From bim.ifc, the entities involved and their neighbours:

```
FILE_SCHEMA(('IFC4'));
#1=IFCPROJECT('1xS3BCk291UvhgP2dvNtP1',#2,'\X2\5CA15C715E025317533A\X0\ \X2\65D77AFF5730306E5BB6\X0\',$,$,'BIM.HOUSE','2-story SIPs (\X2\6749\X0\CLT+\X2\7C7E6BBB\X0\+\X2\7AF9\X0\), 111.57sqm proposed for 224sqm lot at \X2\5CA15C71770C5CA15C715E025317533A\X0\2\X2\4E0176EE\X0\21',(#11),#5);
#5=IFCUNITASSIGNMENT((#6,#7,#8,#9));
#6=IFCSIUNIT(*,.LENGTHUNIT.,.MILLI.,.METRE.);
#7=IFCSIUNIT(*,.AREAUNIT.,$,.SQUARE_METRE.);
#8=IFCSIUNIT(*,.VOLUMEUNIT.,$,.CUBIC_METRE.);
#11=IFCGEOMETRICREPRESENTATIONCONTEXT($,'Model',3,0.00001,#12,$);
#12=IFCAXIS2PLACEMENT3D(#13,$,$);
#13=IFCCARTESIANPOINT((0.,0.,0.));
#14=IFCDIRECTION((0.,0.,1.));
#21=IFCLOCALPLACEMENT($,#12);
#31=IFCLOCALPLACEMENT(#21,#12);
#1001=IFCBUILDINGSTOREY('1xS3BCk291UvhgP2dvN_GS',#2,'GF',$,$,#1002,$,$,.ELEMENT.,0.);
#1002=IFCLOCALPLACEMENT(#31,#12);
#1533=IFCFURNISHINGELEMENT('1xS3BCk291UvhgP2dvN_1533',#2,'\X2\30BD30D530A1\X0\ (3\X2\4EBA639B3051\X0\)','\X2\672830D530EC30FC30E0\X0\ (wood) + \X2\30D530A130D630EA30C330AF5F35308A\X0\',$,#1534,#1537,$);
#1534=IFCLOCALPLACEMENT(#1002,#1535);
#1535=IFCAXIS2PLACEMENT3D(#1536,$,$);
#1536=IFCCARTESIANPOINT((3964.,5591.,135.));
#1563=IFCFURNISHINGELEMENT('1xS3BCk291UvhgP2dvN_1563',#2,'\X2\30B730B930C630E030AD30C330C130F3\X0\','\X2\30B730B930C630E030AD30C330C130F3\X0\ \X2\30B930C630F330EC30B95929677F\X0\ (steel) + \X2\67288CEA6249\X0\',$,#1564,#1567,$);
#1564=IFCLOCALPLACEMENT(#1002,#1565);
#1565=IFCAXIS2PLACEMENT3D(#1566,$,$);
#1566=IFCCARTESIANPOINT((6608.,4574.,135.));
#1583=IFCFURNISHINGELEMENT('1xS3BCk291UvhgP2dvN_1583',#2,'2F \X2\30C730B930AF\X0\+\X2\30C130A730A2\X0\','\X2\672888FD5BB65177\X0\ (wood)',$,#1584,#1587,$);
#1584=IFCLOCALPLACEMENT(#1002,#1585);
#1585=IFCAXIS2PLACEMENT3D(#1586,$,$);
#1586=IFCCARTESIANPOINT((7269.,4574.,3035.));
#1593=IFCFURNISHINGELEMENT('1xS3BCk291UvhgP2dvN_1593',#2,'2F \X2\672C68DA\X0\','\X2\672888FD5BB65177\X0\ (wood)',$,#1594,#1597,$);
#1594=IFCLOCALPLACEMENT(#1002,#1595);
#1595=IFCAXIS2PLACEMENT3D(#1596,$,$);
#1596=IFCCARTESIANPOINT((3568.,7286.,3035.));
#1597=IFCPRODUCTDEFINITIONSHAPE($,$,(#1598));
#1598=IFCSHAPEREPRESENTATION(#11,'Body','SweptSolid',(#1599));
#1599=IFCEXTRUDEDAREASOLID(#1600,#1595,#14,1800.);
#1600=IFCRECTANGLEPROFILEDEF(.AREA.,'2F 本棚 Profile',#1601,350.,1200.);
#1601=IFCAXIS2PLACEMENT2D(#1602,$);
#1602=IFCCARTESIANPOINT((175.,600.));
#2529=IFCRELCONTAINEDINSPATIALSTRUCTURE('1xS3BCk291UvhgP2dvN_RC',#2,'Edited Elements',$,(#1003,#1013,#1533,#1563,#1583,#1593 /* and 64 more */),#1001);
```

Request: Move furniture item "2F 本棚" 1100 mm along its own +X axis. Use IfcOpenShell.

```python
import ifcopenshell
import ifcopenshell.api.geometry
import ifcopenshell.util.placement
import ifcopenshell.util.unit

model = ifcopenshell.open("bim.ifc")
unit_scale = ifcopenshell.util.unit.calculate_unit_scale(model)

item = model.by_guid("1xS3BCk291UvhgP2dvN_1593")
matrix = ifcopenshell.util.placement.get_local_placement(item.ObjectPlacement)
matrix[:3, 3] += matrix[:3, 0] * 1.1 / unit_scale
ifcopenshell.api.geometry.edit_object_placement(model, product=item, matrix=matrix, is_si=False)

print(ifcopenshell.util.placement.get_local_placement(item.ObjectPlacement).round(3) + 0.0)

model.write("bim-out.ifc")
```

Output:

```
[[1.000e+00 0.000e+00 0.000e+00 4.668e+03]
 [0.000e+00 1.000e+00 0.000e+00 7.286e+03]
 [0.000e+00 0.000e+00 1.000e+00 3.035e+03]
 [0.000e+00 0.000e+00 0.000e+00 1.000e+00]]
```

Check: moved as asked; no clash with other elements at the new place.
